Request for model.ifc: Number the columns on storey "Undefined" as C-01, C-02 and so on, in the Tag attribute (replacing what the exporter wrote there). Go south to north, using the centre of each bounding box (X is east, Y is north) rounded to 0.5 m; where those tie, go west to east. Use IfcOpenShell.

First a look at what the model holds.

```python
import ifcopenshell
import ifcopenshell.util.element
import ifcopenshell.util.placement

model = ifcopenshell.open("model.ifc")
print(model.schema)
storey = next(s for s in model.by_type("IfcBuildingStorey") if s.Name == "Undefined")
columns = [e for e in ifcopenshell.util.element.get_decomposition(storey) if e.is_a("IfcColumn")]
for e in sorted(columns, key=lambda e: e.id()):
    origin = ifcopenshell.util.placement.get_local_placement(e.ObjectPlacement)[:3, 3]
    print(e.id(), e.Tag, e.Name, origin.round(2) + 0.0, sep=" | ")
```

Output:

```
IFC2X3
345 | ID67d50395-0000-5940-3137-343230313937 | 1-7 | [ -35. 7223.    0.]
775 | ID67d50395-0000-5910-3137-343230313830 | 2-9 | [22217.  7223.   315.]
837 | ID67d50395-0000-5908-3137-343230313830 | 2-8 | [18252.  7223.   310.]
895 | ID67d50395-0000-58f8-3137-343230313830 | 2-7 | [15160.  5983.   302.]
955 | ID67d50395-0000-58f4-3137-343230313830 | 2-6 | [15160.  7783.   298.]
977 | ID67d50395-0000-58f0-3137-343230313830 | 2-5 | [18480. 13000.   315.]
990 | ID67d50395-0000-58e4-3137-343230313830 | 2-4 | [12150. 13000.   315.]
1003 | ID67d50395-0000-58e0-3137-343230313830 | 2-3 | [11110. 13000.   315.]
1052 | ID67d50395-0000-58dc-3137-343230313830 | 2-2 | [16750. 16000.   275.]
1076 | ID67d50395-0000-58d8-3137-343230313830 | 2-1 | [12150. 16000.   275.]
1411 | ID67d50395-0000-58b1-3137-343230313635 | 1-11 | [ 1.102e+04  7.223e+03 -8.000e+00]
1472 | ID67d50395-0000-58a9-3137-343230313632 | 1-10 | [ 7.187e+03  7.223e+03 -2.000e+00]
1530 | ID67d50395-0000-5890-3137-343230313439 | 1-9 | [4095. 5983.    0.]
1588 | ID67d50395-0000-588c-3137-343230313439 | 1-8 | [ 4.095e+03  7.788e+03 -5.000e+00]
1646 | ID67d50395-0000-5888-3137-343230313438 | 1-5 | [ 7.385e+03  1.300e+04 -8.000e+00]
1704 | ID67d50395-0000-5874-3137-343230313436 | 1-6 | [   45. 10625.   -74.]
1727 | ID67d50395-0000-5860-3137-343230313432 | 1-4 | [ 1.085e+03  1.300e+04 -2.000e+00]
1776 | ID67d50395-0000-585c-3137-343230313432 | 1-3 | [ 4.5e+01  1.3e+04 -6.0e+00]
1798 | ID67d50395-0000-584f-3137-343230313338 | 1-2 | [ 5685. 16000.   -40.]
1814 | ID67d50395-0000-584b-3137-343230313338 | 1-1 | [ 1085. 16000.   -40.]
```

```python
import ifcopenshell
import ifcopenshell.geom
import ifcopenshell.util.element
import ifcopenshell.util.shape

model = ifcopenshell.open("model.ifc")
settings = ifcopenshell.geom.settings()
settings.set("use-world-coords", True)


def centre(element):
    shape = ifcopenshell.geom.create_shape(settings, element)
    return ifcopenshell.util.shape.get_bbox_centroid(shape.geometry)


storey = next(s for s in model.by_type("IfcBuildingStorey") if s.Name == "Undefined")
columns = [e for e in ifcopenshell.util.element.get_decomposition(storey) if e.is_a("IfcColumn")]

# Insertion points can sit at a corner or the storey origin, so sort by the geometry (in metres).
centres = {e: centre(e) for e in columns}
columns.sort(key=lambda e: (round(centres[e][1] / 0.5), centres[e][0]))

for i, e in enumerate(columns, start=1):
    number = f"C-{i:02d}"
    e.Tag = number
    print(e.id(), number)

model.write("model_edited.ifc")
```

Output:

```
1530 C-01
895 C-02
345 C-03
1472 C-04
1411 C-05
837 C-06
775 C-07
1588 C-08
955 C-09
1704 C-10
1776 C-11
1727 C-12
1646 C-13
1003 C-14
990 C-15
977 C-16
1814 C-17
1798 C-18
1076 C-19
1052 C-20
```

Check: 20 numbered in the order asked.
